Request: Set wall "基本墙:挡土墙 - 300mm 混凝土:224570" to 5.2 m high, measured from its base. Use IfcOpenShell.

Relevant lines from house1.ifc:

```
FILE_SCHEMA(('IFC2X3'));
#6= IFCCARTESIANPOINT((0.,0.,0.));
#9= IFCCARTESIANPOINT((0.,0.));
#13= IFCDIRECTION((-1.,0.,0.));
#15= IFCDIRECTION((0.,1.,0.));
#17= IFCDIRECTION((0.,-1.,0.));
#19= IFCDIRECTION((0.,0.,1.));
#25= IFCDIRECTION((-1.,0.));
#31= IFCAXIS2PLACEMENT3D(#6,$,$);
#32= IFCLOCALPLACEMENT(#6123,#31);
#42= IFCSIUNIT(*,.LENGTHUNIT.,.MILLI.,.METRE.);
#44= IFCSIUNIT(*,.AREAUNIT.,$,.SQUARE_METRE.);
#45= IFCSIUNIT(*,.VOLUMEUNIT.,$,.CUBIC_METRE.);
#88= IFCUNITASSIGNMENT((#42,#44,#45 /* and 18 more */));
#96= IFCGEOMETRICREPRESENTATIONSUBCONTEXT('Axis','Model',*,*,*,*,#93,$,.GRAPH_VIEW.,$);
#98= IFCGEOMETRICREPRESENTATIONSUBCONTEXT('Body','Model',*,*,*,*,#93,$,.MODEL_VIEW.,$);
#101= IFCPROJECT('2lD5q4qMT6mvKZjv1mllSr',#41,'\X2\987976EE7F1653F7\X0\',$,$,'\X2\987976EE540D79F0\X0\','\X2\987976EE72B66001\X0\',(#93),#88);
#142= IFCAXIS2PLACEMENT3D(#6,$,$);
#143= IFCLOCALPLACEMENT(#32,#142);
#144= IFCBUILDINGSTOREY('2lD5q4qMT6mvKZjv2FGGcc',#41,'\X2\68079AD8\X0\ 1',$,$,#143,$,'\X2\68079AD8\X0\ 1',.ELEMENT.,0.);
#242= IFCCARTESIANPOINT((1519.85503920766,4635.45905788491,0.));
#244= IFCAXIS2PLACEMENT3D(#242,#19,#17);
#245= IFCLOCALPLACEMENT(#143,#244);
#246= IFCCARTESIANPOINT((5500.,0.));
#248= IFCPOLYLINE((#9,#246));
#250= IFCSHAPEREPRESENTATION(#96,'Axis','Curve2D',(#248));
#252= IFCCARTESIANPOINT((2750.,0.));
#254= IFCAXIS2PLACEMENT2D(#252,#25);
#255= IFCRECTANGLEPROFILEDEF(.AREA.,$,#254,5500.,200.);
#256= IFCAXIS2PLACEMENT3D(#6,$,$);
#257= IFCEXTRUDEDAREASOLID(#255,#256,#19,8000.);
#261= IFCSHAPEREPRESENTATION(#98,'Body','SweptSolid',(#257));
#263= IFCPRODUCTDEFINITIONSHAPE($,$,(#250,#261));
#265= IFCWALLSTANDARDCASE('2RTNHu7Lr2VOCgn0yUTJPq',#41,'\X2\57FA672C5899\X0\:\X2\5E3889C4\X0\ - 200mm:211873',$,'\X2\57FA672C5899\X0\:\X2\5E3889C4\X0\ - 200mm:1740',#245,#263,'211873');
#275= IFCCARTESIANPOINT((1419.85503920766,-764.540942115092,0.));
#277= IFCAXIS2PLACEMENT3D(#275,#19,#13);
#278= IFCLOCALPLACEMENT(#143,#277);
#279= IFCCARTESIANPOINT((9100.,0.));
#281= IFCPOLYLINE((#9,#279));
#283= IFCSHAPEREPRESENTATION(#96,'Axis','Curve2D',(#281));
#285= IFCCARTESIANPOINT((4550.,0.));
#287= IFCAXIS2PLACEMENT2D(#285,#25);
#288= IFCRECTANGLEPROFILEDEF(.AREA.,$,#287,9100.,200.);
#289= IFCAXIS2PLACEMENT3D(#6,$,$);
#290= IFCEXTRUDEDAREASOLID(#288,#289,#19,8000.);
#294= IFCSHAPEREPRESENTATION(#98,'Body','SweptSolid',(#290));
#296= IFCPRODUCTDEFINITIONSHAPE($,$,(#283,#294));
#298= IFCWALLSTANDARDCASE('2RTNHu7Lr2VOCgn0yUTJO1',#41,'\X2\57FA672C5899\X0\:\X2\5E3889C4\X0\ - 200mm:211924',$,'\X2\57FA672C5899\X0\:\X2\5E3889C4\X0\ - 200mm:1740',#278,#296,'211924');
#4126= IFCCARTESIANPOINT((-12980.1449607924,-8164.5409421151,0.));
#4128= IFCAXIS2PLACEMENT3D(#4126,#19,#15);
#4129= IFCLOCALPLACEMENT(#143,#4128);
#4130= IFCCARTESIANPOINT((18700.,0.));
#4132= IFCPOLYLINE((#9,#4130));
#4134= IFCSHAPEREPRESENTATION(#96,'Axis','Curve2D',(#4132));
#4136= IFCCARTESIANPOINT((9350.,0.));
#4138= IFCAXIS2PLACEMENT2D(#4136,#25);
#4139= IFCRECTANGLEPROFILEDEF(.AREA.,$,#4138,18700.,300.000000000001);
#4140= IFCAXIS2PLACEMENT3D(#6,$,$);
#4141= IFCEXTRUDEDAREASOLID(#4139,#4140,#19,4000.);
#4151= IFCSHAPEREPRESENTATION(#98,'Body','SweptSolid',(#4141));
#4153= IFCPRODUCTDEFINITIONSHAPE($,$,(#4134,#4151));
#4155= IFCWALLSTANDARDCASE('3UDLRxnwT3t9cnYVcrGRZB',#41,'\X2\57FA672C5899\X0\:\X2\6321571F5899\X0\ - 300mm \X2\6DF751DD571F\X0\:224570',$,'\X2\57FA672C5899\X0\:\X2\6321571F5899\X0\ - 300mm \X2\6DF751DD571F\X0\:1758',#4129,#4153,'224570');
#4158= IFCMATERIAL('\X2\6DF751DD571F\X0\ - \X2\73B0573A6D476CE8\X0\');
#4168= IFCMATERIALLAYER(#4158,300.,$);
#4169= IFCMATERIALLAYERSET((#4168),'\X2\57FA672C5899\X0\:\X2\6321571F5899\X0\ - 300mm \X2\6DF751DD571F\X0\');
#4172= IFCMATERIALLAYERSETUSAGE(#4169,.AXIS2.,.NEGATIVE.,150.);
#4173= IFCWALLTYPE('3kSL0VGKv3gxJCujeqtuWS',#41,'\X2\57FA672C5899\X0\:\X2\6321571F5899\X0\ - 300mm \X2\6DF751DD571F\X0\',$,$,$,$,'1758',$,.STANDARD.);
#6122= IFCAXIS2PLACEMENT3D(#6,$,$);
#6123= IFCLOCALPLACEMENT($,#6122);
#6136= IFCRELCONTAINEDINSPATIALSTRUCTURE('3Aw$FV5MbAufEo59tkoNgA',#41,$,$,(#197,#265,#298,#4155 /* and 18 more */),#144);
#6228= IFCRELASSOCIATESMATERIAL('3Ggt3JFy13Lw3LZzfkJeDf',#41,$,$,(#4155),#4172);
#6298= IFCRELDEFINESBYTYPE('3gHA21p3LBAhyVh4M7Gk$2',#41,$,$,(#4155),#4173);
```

```python
import ifcopenshell
import ifcopenshell.geom
import ifcopenshell.util.representation
import ifcopenshell.util.shape
import ifcopenshell.util.unit

model = ifcopenshell.open("house1.ifc")
unit_scale = ifcopenshell.util.unit.calculate_unit_scale(model)
settings = ifcopenshell.geom.settings()


def volume(element):
    """Net volume in cubic metres, openings subtracted."""
    shape = ifcopenshell.geom.create_shape(settings, element)
    return ifcopenshell.util.shape.get_volume(shape.geometry)


wall = model.by_id(4155)
before = volume(wall)

body = ifcopenshell.util.representation.get_representation(wall, "Model", "Body")
solid = body.Items[0]
old_height = solid.Depth
solid.Depth = 5.2 / unit_scale
after = volume(wall)

print(f"height {old_height:g} -> {solid.Depth:g}, volume {before:.3f} -> {after:.3f} m3")

model.write("house1_updated.ifc")
```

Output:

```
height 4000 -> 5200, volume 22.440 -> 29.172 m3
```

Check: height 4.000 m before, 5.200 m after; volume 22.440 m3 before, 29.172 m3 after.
